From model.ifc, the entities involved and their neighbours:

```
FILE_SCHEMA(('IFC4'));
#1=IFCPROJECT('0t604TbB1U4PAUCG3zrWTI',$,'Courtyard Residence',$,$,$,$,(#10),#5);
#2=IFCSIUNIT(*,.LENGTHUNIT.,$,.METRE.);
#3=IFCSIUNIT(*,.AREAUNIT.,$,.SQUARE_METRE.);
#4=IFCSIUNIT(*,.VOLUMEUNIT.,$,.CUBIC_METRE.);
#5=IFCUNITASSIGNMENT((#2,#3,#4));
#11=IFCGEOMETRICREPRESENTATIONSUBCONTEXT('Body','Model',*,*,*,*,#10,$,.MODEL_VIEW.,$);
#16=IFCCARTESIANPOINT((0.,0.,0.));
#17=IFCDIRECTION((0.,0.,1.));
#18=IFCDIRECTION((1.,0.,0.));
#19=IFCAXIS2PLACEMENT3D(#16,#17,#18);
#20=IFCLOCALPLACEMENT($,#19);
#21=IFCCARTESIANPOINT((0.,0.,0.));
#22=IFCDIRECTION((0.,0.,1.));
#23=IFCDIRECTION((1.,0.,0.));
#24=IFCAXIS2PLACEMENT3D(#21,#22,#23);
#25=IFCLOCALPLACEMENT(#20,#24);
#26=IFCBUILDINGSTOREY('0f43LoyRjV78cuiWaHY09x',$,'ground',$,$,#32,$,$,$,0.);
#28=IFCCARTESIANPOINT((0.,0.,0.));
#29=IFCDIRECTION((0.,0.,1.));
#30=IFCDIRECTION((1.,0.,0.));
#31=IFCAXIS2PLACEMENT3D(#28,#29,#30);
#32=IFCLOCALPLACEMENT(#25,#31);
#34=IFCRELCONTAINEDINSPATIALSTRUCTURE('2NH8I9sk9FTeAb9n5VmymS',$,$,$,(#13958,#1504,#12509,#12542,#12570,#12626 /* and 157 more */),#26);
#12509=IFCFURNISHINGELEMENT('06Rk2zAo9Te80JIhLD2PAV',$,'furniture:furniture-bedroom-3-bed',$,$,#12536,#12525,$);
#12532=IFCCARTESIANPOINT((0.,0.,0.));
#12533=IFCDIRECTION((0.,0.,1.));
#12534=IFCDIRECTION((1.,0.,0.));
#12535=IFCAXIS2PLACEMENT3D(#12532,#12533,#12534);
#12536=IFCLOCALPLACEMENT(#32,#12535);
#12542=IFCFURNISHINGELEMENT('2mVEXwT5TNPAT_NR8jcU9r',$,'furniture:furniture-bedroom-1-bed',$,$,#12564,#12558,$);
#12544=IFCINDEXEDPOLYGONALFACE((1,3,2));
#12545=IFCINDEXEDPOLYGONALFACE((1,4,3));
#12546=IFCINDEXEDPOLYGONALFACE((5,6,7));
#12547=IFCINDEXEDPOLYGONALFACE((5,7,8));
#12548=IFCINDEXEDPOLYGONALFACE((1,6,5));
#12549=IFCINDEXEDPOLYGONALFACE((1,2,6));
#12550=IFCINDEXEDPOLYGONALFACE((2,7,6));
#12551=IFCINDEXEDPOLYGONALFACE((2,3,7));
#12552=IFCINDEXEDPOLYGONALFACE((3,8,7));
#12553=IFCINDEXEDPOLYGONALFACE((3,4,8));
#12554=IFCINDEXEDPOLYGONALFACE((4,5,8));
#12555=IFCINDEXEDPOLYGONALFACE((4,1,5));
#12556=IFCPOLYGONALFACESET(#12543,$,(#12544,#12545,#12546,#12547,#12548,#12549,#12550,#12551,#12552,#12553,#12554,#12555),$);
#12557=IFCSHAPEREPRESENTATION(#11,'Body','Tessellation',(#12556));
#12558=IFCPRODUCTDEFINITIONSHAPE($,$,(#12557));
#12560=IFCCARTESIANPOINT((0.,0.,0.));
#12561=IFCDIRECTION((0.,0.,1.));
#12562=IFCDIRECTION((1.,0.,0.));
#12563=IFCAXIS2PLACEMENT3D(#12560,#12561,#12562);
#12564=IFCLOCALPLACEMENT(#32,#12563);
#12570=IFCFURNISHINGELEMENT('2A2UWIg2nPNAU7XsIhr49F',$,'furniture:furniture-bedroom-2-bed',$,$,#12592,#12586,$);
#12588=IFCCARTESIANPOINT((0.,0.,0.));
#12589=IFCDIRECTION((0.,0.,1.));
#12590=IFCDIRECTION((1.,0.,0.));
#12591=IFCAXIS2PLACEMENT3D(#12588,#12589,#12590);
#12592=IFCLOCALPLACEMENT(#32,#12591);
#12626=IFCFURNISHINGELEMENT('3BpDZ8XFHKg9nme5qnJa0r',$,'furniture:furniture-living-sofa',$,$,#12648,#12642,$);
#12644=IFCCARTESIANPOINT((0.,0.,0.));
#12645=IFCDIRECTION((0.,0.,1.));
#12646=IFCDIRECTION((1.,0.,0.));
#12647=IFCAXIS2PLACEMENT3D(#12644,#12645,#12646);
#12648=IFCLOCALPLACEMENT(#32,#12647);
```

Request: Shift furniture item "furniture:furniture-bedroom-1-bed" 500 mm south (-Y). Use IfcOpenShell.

```python
import ifcopenshell
import ifcopenshell.api.geometry
import ifcopenshell.util.placement
import ifcopenshell.util.unit

model = ifcopenshell.open("model.ifc")
unit_scale = ifcopenshell.util.unit.calculate_unit_scale(model)

item = model.by_id(12542)
matrix = ifcopenshell.util.placement.get_local_placement(item.ObjectPlacement)
matrix[1, 3] -= 0.5 / unit_scale
ifcopenshell.api.geometry.edit_object_placement(model, product=item, matrix=matrix, is_si=False)

print(ifcopenshell.util.placement.get_local_placement(item.ObjectPlacement).round(3) + 0.0)

model.write("model_v2.ifc")
```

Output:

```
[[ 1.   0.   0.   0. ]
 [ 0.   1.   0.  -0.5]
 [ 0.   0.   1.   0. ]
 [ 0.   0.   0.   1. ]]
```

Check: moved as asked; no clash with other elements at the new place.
